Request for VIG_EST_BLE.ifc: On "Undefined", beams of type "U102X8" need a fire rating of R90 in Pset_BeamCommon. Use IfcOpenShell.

First a look at what the model holds.

```python
import ifcopenshell
import ifcopenshell.util.element

model = ifcopenshell.open("VIG_EST_BLE.ifc")
print(model.schema)
storey = next(s for s in model.by_type("IfcBuildingStorey") if s.Name == "Undefined")
beams = [e for e in ifcopenshell.util.element.get_decomposition(storey) if e.is_a("IfcBeam")]
seen = {}
for e in beams:
    element_type = ifcopenshell.util.element.get_type(e)
    key = (element_type.Name if element_type != e and element_type else None, ifcopenshell.util.element.get_pset(e, "Pset_BeamCommon", "FireRating"))
    seen[key] = seen.get(key, 0) + 1
for (name, value), count in sorted(seen.items(), key=str):
    print(count, "x", name, "|", value)
```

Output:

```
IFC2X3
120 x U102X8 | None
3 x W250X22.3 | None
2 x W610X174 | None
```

```python
import ifcopenshell
import ifcopenshell.api.pset
import ifcopenshell.util.element

model = ifcopenshell.open("VIG_EST_BLE.ifc")

storey = next(s for s in model.by_type("IfcBuildingStorey") if s.Name == "Undefined")
beams = [e for e in ifcopenshell.util.element.get_decomposition(storey) if e.is_a("IfcBeam")]

count = 0
for e in beams:
    element_type = ifcopenshell.util.element.get_type(e)
    if element_type in (None, e) or element_type.Name != "U102X8":
        continue
    found = ifcopenshell.util.element.get_pset(e, "Pset_BeamCommon", should_inherit=False)
    if found:
        pset = model.by_id(found["id"])
        if len(ifcopenshell.util.element.get_elements_by_pset(pset)) > 1:
            pset = ifcopenshell.api.pset.unshare_pset(model, products=[e], pset=pset)[0]
    else:
        pset = ifcopenshell.api.pset.add_pset(model, product=e, name="Pset_BeamCommon")
    ifcopenshell.api.pset.edit_pset(model, pset=pset, properties={"FireRating": "R90"})
    count += 1

print(count, "beams updated")

model.write("VIG_EST_BLE_v2.ifc")
```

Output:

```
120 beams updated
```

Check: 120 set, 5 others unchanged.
